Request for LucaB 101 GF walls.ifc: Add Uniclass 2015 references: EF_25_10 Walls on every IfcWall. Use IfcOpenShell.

First a look at what the model holds.

```python
import ifcopenshell

model = ifcopenshell.open("LucaB 101 GF walls.ifc")
print(model.schema)
print("classifications:", [c.Name for c in model.by_type("IfcClassification")])
for ifc_class in ("IfcDoor", "IfcRoof", "IfcStair", "IfcWall", "IfcWindow"):
    print(ifc_class, len(model.by_type(ifc_class)))
```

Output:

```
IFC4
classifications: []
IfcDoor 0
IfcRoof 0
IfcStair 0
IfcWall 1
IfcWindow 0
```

```python
import ifcopenshell
import ifcopenshell.api.classification

model = ifcopenshell.open("LucaB 101 GF walls.ifc")

system = ifcopenshell.api.classification.add_classification(model, classification="Uniclass 2015")

codes = {
    "IfcWall": ("EF_25_10", "Walls"),
}
for ifc_class, (code, name) in codes.items():
    products = model.by_type(ifc_class)
    ifcopenshell.api.classification.add_reference(
        model, products=products, classification=system, identification=code, name=name
    )
    print(code, len(products))

model.write("LucaB 101 GF walls_v2.ifc")
```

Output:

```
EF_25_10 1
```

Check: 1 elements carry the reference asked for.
